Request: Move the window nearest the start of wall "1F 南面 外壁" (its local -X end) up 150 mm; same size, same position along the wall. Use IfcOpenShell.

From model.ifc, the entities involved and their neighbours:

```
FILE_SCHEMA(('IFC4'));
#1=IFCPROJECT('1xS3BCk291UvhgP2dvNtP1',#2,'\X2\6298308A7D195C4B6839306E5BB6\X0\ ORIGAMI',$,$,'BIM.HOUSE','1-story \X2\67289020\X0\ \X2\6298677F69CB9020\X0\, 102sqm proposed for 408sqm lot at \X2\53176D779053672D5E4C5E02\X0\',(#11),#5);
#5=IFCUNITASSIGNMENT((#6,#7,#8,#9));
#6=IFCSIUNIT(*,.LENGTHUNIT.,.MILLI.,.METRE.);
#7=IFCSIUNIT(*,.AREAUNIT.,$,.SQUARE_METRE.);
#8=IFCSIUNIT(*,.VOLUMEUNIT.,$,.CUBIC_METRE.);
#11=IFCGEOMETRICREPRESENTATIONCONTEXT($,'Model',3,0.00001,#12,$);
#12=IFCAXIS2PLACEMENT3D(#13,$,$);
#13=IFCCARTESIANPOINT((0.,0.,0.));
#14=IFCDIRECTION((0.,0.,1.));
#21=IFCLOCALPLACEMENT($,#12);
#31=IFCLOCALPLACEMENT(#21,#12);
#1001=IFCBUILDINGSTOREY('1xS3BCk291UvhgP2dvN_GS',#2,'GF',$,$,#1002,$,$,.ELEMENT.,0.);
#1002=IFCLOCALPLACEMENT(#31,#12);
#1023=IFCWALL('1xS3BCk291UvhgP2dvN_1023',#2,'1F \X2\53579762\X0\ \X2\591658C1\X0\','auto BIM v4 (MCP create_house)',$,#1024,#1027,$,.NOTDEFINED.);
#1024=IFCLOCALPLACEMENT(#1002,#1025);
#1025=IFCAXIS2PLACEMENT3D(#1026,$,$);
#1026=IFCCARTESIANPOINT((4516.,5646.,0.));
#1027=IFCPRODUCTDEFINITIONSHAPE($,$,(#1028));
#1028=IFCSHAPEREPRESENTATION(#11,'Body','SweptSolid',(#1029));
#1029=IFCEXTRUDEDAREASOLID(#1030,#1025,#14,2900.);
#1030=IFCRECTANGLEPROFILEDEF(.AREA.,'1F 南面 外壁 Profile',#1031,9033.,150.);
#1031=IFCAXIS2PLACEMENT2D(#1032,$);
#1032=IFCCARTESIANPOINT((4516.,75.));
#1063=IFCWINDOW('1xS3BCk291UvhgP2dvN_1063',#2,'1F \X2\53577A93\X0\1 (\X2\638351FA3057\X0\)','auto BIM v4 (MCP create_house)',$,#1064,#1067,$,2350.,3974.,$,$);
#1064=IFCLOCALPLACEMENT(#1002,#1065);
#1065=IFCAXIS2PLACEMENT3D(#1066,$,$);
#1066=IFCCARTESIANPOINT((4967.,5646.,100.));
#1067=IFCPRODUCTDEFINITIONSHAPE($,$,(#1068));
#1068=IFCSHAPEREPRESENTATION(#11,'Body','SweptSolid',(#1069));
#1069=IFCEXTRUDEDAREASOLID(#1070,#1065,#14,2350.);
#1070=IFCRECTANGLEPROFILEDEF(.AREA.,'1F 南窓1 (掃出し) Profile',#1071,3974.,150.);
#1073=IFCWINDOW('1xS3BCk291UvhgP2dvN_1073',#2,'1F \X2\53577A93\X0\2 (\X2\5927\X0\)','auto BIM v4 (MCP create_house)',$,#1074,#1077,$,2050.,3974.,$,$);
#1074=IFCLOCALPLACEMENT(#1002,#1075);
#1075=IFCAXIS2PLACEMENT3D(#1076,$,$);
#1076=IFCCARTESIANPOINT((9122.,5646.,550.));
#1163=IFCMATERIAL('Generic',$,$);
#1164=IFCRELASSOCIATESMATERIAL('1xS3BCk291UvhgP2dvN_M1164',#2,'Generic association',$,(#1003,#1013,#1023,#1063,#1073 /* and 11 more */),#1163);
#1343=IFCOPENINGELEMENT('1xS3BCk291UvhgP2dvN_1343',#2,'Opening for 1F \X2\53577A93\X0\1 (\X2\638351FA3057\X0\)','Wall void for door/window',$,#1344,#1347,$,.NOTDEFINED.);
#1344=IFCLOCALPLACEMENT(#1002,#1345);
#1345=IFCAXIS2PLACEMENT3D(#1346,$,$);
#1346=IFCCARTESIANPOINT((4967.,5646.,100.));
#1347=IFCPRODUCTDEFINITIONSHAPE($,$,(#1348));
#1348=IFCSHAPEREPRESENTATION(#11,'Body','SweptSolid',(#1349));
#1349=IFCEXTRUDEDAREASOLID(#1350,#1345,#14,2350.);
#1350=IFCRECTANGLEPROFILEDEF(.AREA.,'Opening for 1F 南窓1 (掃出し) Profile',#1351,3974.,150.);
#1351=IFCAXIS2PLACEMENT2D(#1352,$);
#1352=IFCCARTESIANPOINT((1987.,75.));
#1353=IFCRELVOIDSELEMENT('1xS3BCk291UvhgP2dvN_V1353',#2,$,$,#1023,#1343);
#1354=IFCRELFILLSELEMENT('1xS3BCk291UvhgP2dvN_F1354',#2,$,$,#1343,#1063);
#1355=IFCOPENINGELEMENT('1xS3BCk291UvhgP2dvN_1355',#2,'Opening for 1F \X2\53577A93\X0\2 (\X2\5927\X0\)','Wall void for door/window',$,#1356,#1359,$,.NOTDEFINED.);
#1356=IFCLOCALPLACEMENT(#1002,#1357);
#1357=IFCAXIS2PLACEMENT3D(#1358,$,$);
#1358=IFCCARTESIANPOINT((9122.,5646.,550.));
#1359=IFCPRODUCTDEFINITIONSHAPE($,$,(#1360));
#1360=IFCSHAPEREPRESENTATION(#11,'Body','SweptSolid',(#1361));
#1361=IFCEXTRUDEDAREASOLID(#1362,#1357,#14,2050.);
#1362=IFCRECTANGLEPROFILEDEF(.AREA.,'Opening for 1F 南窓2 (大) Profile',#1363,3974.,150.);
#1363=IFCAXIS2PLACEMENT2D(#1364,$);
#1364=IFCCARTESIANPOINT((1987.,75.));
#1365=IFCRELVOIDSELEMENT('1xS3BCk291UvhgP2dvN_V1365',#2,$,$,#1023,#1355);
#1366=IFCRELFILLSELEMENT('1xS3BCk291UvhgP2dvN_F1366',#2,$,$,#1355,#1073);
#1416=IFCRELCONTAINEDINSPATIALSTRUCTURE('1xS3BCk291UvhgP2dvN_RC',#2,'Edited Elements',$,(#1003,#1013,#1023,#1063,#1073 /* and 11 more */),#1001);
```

```python
import numpy as np
import ifcopenshell
import ifcopenshell.api.geometry
import ifcopenshell.util.placement
import ifcopenshell.util.unit

model = ifcopenshell.open("model.ifc")
unit_scale = ifcopenshell.util.unit.calculate_unit_scale(model)

window = model.by_guid("1xS3BCk291UvhgP2dvN_1063")
opening = window.FillsVoids[0].RelatingOpeningElement
dz = 150.0

shift = np.array([0.0, 0.0, dz])
# The window is not placed relative to its opening, so move both.
for product in (opening, window):
    matrix = ifcopenshell.util.placement.get_local_placement(product.ObjectPlacement)
    matrix[:3, 3] += shift
    ifcopenshell.api.geometry.edit_object_placement(model, product=product, matrix=matrix, is_si=False)

print(f"moved by {dz * unit_scale:+.3f} m")

model.write("model_v2.ifc")
```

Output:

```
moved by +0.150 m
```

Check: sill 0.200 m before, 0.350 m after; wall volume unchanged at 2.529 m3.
